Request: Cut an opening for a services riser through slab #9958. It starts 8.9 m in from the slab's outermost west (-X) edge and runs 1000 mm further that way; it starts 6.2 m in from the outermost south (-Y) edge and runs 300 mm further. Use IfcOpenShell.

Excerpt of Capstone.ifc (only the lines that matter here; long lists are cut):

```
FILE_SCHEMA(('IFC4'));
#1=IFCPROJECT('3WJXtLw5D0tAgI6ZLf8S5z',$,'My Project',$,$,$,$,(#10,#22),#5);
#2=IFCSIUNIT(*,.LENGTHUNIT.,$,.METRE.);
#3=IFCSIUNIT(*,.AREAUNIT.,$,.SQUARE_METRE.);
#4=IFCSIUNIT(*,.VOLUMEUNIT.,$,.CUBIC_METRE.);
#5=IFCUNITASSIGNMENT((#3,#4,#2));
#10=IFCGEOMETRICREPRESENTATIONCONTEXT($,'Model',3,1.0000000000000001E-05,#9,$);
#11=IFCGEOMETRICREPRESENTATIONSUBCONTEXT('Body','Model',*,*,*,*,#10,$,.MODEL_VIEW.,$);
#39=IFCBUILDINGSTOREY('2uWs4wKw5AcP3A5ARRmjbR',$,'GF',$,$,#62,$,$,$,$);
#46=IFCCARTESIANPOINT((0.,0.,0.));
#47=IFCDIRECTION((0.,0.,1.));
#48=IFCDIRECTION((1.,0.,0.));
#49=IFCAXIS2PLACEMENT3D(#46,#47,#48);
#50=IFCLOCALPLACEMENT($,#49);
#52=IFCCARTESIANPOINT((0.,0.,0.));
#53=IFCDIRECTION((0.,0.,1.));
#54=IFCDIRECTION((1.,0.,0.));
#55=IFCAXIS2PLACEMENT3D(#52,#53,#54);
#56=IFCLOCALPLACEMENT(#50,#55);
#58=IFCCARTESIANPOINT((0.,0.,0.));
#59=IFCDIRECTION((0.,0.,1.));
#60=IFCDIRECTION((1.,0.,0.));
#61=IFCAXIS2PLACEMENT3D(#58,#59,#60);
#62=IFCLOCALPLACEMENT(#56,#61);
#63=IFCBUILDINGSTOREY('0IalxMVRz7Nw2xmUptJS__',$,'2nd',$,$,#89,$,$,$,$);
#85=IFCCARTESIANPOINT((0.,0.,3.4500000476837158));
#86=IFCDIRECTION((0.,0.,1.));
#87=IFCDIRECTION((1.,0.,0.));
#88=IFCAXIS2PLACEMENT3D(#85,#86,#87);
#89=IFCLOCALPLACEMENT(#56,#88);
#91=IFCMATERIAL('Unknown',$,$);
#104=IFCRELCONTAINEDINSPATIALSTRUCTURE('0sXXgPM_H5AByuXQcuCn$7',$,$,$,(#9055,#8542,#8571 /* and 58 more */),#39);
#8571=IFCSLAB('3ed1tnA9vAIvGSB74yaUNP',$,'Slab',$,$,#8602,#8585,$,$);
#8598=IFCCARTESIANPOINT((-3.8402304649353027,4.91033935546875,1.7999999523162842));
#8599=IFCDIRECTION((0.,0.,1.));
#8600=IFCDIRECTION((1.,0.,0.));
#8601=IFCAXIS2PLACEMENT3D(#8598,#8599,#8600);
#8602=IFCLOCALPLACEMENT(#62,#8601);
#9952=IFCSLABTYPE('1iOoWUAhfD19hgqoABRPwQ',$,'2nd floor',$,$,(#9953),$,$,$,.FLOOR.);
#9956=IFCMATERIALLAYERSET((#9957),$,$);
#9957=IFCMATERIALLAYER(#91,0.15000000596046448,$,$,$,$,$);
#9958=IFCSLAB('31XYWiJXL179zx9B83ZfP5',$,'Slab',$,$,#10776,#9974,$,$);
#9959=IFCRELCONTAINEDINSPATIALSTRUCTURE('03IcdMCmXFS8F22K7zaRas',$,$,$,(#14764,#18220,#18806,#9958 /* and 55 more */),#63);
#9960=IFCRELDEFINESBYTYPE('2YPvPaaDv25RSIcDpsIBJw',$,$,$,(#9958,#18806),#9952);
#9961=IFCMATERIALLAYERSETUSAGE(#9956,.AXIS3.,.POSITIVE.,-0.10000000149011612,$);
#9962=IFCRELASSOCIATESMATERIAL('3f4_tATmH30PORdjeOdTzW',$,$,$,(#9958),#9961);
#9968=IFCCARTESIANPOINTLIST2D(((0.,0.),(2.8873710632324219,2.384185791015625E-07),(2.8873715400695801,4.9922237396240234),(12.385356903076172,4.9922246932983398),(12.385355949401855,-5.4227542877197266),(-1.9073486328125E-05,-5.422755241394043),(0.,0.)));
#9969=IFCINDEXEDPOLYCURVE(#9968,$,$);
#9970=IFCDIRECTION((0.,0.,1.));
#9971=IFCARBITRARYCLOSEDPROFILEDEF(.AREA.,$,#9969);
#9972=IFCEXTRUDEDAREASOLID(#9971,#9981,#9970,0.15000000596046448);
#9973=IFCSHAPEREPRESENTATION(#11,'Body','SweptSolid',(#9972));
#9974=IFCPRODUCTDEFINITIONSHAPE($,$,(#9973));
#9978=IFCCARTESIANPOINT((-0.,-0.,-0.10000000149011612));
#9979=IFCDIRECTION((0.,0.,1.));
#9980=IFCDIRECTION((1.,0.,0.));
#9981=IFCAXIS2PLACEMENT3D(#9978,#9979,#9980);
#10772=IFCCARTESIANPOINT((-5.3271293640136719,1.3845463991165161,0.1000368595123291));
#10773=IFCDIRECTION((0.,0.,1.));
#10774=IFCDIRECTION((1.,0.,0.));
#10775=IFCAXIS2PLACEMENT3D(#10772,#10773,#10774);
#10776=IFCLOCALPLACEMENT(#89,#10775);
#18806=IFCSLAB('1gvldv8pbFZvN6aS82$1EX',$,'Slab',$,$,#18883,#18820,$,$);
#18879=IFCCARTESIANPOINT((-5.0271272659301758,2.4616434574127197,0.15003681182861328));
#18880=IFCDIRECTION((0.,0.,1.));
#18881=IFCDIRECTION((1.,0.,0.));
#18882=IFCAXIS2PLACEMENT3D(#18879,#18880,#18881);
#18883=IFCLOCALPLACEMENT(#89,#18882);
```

```python
import numpy as np
import ifcopenshell
import ifcopenshell.api.feature
import ifcopenshell.api.geometry
import ifcopenshell.api.root
import ifcopenshell.geom
import ifcopenshell.util.placement
import ifcopenshell.util.representation
import ifcopenshell.util.shape
import ifcopenshell.util.unit

model = ifcopenshell.open("Capstone.ifc")
unit_scale = ifcopenshell.util.unit.calculate_unit_scale(model)
settings = ifcopenshell.geom.settings()


def volume(element):
    """Net volume in cubic metres, openings subtracted."""
    shape = ifcopenshell.geom.create_shape(settings, element)
    return ifcopenshell.util.shape.get_volume(shape.geometry)


slab = model.by_id(9958)
before = volume(slab)

# Extent in the slab's own axes, in metres. The edges named are its -X and -Y sides.
slab_shape = ifcopenshell.geom.create_shape(settings, slab)
vertices = ifcopenshell.util.shape.get_vertices(slab_shape.geometry)
x_min, y_min, bottom = vertices.min(axis=0)
top = vertices[:, 2].max()

opening = ifcopenshell.api.root.create_entity(model, ifc_class="IfcOpeningElement", name="Services riser opening", predefined_type="OPENING")
context = ifcopenshell.util.representation.get_context(model, "Model", "Body", "MODEL_VIEW")
width, depth = 1, 0.3
outline = [(0.0, 0.0), (width, 0.0), (width, depth), (0.0, depth), (0.0, 0.0)]
# Overshoot both faces by 50 mm so the cut is clean.
shape = ifcopenshell.api.geometry.add_slab_representation(
    model, context=context, depth=top - bottom + 0.1, polyline=outline
)
ifcopenshell.api.geometry.assign_representation(model, product=opening, representation=shape)

matrix = ifcopenshell.util.placement.get_local_placement(slab.ObjectPlacement)
matrix[:, 3] = matrix @ np.append(np.array([x_min + 8.9, y_min + 6.2, bottom - 0.05]) / unit_scale, 1.0)
ifcopenshell.api.geometry.edit_object_placement(model, product=opening, matrix=matrix, is_si=False)
ifcopenshell.api.feature.add_feature(model, feature=opening, element=slab)

after = volume(slab)

print(f"slab volume {before:.3f} -> {after:.3f} m3")

model.write("Capstone_v2.ifc")
```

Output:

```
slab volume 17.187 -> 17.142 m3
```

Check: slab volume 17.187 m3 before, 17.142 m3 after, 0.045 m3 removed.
